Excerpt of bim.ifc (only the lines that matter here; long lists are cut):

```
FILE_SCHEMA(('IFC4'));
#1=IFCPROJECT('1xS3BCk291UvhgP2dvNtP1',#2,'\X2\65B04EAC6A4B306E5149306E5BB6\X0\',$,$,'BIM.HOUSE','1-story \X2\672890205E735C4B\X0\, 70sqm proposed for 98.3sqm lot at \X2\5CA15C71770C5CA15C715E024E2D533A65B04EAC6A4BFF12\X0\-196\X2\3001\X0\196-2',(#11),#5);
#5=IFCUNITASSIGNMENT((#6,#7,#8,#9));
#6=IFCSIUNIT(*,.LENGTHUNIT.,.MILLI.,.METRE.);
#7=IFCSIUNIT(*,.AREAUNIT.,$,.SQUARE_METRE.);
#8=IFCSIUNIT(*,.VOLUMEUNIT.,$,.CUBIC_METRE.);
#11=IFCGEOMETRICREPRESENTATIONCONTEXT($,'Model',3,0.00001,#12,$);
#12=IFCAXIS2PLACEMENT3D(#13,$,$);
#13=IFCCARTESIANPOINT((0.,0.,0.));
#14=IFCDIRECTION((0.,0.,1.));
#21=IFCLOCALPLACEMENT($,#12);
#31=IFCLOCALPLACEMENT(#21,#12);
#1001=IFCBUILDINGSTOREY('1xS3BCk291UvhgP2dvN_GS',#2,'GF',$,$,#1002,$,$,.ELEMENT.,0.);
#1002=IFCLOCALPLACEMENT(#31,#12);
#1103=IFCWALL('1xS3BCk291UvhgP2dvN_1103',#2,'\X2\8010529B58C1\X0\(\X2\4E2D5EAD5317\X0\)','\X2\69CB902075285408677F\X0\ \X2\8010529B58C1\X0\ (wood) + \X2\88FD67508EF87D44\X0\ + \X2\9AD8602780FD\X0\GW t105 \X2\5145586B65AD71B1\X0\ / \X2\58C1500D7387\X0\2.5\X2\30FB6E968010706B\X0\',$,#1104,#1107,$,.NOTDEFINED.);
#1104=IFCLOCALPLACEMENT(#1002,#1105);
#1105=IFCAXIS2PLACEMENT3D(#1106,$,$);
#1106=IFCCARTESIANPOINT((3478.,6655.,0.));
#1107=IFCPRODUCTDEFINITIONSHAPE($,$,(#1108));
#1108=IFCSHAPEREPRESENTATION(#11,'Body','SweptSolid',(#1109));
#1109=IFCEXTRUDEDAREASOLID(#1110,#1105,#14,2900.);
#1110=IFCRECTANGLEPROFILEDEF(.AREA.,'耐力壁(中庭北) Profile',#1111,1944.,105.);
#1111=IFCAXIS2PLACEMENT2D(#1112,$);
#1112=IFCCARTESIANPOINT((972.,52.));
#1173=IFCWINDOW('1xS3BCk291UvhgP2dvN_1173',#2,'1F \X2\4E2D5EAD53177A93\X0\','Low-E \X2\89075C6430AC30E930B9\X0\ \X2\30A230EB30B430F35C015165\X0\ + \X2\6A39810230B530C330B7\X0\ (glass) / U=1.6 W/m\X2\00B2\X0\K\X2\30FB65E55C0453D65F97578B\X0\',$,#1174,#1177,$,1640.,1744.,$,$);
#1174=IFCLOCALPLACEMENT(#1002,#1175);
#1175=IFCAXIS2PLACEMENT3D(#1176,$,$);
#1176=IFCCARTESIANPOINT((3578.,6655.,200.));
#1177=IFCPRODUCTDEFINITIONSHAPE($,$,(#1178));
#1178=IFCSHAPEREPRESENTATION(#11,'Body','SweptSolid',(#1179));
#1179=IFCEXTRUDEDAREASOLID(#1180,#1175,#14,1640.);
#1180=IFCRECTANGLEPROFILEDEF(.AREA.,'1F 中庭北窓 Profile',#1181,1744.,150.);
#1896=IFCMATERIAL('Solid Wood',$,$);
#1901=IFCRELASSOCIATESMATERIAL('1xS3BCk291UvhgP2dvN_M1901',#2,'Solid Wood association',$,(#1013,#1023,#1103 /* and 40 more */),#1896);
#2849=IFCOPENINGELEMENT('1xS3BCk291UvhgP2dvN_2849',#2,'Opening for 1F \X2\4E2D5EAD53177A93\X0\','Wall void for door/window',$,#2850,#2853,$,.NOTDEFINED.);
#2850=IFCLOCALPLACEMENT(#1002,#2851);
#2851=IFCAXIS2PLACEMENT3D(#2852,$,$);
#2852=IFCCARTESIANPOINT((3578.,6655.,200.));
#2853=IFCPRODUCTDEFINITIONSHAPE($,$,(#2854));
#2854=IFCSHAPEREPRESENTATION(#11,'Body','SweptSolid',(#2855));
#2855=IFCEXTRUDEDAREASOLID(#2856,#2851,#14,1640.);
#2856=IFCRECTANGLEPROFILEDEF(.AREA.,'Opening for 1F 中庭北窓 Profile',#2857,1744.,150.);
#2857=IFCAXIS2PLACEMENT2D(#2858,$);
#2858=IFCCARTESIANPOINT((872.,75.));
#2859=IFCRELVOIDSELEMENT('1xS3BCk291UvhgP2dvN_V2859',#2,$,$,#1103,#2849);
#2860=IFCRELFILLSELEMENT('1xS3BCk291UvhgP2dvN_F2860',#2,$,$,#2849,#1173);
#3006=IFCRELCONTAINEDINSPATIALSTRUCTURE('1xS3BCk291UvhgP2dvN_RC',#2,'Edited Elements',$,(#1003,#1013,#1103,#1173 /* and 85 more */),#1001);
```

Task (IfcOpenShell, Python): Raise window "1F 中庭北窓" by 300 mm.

```python
import numpy as np
import ifcopenshell
import ifcopenshell.api.geometry
import ifcopenshell.util.placement
import ifcopenshell.util.unit

model = ifcopenshell.open("bim.ifc")
unit_scale = ifcopenshell.util.unit.calculate_unit_scale(model)

window = model.by_guid("1xS3BCk291UvhgP2dvN_1173")
opening = window.FillsVoids[0].RelatingOpeningElement
dz = 300.0

shift = np.array([0.0, 0.0, dz])
# The window is not placed relative to its opening, so move both.
for product in (opening, window):
    matrix = ifcopenshell.util.placement.get_local_placement(product.ObjectPlacement)
    matrix[:3, 3] += shift
    ifcopenshell.api.geometry.edit_object_placement(model, product=product, matrix=matrix, is_si=False)

print(f"moved by {dz * unit_scale:+.3f} m")

model.write("bim_v2.ifc")
```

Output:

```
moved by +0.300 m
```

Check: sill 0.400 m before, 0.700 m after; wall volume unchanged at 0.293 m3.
